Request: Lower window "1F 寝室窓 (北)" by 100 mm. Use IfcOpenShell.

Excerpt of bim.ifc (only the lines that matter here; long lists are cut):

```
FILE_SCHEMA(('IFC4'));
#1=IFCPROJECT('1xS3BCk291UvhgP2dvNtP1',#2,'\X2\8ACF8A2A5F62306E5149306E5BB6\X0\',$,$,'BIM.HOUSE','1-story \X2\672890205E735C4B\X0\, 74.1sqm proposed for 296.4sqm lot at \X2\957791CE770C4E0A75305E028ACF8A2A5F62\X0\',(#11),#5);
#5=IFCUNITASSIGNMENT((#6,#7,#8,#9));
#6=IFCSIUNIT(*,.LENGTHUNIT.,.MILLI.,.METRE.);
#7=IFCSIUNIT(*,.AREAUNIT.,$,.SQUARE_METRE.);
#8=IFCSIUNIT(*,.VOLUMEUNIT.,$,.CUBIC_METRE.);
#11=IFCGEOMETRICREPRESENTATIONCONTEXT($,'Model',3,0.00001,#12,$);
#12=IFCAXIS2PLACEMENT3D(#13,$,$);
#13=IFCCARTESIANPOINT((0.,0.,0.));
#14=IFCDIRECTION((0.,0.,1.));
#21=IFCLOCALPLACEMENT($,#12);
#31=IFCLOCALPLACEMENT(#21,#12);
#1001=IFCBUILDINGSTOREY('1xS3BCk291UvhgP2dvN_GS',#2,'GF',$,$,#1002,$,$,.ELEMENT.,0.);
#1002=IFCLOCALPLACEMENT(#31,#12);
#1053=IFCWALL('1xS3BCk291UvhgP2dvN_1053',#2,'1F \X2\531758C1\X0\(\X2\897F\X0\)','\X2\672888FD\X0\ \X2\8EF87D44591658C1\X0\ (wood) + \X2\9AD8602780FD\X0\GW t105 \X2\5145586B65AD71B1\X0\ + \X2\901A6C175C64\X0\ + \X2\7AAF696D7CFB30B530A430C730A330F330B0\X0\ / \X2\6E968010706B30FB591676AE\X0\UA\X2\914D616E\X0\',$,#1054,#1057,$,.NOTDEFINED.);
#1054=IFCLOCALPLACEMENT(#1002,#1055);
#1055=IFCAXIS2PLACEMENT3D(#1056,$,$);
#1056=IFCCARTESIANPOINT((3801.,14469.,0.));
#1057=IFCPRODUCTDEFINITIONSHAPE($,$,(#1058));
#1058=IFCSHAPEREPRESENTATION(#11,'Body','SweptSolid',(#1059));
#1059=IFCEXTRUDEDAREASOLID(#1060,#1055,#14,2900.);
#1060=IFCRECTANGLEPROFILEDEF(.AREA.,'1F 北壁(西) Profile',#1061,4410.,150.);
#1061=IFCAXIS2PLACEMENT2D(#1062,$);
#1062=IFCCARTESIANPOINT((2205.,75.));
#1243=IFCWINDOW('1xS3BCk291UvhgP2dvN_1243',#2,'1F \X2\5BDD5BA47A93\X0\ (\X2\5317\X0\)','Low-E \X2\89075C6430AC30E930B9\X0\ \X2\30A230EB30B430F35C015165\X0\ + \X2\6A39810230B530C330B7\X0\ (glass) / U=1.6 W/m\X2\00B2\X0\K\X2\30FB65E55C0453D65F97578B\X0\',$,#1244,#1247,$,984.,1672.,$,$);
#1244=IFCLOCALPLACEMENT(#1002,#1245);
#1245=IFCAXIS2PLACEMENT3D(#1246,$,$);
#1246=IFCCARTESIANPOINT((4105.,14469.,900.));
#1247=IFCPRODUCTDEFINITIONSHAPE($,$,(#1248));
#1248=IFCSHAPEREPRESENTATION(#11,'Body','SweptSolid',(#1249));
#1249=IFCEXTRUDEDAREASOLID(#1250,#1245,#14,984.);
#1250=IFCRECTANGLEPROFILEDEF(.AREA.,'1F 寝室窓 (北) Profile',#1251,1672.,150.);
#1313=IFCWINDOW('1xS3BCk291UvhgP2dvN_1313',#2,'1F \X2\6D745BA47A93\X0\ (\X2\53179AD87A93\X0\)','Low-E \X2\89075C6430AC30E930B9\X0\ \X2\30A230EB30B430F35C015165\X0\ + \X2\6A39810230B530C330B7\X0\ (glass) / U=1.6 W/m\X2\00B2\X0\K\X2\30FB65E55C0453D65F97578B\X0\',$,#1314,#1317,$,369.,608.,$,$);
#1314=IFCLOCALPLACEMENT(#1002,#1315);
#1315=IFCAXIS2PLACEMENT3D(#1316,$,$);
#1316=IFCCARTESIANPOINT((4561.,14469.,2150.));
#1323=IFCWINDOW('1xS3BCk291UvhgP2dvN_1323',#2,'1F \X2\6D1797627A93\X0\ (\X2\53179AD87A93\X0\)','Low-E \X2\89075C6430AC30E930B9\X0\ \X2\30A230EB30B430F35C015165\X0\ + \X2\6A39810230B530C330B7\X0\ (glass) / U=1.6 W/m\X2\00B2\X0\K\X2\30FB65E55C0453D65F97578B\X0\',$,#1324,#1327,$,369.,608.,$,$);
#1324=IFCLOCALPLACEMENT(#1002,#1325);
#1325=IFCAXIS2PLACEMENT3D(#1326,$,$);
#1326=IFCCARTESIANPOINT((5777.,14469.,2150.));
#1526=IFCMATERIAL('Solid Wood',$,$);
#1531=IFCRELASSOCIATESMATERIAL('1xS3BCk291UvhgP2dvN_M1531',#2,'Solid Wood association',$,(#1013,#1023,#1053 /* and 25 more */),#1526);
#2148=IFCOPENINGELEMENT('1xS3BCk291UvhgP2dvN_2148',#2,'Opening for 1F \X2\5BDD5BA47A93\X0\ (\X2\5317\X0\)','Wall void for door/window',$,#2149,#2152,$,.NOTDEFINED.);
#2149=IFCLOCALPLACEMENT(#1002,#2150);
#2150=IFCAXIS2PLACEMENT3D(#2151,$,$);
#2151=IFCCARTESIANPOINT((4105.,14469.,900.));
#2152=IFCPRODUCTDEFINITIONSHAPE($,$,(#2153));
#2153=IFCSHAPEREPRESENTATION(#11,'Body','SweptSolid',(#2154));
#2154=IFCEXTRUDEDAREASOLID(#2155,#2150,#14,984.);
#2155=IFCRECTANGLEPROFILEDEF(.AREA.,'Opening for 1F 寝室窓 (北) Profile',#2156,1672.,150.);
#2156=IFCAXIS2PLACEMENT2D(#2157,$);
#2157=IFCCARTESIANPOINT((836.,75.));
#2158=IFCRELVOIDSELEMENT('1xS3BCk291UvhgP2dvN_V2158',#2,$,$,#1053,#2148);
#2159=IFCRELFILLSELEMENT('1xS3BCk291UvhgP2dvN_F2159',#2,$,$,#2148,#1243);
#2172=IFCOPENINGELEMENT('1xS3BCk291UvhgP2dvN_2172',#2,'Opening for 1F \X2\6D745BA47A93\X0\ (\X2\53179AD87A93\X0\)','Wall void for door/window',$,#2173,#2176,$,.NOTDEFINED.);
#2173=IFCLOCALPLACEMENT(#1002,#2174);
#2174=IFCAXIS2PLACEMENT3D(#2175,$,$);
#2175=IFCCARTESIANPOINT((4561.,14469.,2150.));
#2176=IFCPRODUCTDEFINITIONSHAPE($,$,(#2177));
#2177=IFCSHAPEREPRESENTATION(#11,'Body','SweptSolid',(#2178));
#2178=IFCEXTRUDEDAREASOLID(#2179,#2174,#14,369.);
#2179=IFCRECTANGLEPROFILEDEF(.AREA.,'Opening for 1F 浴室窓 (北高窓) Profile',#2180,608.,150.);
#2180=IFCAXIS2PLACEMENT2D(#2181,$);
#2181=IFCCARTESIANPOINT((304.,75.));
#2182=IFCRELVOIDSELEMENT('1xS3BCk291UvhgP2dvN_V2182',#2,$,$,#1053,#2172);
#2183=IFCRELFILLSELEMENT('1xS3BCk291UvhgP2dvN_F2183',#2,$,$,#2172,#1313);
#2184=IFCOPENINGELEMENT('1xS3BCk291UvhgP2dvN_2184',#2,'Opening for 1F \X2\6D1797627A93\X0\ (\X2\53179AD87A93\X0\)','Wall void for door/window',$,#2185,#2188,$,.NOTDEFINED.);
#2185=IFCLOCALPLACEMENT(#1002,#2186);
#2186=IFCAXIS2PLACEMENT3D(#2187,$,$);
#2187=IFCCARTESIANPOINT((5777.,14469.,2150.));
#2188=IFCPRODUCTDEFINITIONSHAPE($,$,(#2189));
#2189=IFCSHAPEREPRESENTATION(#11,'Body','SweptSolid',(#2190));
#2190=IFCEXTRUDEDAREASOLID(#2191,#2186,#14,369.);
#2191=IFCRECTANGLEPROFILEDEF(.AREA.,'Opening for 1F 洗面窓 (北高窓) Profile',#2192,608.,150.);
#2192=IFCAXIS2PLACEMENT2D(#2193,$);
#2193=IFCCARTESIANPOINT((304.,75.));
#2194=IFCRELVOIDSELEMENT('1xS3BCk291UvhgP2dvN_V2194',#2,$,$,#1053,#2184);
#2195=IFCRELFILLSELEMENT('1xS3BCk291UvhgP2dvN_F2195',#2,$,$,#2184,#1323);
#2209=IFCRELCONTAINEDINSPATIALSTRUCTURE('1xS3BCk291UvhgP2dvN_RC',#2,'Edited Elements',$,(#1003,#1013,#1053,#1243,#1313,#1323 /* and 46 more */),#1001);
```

```python
import numpy as np
import ifcopenshell
import ifcopenshell.api.geometry
import ifcopenshell.util.placement
import ifcopenshell.util.unit

model = ifcopenshell.open("bim.ifc")
unit_scale = ifcopenshell.util.unit.calculate_unit_scale(model)

window = model.by_guid("1xS3BCk291UvhgP2dvN_1243")
opening = window.FillsVoids[0].RelatingOpeningElement
dz = -0.1 / unit_scale

shift = np.array([0.0, 0.0, dz])
# The window is not placed relative to its opening, so move both.
for product in (opening, window):
    matrix = ifcopenshell.util.placement.get_local_placement(product.ObjectPlacement)
    matrix[:3, 3] += shift
    ifcopenshell.api.geometry.edit_object_placement(model, product=product, matrix=matrix, is_si=False)

print(f"moved by {dz * unit_scale:+.3f} m")

model.write("bim_v2.ifc")
```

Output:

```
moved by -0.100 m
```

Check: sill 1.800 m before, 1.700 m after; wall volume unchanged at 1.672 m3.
